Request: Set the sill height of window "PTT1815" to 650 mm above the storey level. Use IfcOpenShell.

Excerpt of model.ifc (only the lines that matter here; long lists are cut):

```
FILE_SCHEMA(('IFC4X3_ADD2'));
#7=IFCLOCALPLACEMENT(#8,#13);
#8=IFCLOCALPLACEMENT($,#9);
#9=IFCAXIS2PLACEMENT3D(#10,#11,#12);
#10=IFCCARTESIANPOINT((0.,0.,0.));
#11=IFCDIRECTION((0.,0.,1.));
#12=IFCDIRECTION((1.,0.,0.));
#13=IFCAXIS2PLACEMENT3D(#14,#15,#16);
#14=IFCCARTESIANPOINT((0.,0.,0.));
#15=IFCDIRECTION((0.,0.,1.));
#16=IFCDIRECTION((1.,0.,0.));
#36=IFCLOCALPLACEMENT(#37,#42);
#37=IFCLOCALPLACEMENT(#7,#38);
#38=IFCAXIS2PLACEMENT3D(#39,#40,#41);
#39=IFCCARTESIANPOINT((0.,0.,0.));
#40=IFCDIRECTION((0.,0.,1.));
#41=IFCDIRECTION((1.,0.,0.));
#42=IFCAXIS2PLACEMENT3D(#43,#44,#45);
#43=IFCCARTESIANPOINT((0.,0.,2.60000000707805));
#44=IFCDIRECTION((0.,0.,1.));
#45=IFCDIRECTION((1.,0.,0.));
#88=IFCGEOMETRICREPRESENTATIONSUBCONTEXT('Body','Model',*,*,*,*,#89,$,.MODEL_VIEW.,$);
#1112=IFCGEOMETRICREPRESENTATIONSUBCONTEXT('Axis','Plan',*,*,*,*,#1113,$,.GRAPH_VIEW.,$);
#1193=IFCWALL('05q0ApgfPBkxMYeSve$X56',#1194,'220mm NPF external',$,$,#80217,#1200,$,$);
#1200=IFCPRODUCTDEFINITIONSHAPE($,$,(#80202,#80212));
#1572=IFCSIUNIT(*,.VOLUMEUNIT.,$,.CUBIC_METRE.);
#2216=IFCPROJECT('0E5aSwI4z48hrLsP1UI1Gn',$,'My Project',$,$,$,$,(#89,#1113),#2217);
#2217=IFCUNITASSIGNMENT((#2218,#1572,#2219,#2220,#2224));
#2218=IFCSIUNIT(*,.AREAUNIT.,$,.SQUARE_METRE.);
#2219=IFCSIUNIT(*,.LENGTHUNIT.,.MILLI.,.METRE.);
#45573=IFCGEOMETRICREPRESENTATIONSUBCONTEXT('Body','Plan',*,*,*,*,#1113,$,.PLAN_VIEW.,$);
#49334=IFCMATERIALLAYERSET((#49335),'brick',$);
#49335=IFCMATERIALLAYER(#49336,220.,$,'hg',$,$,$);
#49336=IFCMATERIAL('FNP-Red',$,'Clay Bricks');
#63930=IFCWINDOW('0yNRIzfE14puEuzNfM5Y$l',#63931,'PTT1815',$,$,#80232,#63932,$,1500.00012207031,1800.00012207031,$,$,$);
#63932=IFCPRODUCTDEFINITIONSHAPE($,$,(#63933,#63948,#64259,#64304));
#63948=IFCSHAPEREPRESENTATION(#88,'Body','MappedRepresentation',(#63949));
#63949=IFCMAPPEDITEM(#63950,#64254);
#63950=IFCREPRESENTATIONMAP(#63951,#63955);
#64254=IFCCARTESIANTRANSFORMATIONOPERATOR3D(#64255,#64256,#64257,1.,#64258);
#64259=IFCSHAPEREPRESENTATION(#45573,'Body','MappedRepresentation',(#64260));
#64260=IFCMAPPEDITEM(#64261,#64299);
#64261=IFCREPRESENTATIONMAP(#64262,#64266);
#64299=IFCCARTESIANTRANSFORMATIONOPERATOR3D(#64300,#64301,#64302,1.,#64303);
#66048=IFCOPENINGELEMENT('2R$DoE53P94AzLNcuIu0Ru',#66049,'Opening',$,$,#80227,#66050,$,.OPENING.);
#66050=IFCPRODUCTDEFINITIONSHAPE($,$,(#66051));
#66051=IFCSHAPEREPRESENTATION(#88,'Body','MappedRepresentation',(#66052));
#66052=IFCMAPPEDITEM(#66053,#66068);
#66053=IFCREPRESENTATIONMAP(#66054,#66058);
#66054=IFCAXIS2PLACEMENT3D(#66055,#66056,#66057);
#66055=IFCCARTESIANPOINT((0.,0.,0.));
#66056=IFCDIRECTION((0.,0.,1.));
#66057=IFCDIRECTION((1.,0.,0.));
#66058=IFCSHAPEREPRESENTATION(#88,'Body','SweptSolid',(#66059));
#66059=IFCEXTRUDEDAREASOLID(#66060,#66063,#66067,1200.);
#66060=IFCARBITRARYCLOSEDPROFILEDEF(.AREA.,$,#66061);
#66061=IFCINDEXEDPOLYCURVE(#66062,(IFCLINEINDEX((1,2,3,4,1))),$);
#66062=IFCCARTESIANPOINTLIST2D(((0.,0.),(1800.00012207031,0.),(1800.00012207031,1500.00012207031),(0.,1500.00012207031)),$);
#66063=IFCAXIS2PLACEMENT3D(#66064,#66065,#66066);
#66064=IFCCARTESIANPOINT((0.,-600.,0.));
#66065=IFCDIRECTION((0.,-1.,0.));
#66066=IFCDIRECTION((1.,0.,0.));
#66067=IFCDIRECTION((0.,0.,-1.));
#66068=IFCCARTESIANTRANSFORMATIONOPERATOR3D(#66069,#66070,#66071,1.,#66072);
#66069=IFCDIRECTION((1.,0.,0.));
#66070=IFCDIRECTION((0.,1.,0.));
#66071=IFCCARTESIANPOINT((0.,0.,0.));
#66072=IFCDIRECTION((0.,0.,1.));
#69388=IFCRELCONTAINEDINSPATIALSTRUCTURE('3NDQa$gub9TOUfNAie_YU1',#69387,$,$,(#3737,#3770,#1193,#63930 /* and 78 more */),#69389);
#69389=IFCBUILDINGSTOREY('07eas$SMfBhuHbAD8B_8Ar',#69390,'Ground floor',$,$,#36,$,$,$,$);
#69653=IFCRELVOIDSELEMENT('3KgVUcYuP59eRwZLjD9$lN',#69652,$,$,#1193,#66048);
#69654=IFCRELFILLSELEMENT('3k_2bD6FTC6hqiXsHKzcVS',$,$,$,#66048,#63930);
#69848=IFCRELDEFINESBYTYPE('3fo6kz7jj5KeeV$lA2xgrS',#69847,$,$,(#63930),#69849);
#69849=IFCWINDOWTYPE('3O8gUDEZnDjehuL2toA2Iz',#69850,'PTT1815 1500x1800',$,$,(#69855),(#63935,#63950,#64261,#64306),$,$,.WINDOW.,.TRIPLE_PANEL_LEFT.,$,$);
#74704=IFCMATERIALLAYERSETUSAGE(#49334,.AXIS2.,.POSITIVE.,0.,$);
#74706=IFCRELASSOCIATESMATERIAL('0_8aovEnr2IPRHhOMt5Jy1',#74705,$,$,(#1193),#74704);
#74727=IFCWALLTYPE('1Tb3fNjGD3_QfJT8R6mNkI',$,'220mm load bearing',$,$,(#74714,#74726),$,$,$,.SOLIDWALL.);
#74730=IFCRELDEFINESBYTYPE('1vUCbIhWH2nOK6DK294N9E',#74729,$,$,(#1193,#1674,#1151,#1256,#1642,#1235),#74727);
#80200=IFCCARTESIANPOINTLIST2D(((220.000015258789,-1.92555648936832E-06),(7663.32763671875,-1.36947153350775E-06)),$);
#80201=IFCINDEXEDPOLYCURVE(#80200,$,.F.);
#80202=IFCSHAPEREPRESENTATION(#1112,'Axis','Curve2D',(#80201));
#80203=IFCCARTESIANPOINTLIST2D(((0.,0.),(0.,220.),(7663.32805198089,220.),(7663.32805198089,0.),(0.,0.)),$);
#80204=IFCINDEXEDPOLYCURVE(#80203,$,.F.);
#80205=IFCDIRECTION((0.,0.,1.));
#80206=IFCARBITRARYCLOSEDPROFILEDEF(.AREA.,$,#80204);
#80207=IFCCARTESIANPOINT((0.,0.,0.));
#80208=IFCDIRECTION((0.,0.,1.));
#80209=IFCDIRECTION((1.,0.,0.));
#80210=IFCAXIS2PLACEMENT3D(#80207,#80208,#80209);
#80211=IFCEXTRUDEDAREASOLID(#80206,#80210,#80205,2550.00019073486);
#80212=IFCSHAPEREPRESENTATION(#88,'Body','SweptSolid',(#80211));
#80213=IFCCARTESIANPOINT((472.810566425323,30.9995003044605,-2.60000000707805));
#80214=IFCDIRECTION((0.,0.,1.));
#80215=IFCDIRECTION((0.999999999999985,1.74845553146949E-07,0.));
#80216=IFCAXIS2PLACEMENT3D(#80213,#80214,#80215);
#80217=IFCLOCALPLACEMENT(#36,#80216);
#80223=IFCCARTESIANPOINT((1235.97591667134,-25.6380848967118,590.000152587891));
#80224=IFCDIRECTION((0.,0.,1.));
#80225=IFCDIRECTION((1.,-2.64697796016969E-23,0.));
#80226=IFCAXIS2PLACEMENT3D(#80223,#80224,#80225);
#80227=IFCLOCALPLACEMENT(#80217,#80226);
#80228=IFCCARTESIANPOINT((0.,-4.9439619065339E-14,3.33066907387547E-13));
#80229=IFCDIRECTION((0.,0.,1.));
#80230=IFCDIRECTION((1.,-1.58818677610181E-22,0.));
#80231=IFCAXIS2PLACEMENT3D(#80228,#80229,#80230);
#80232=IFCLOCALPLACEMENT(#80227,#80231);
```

```python
import numpy as np
import ifcopenshell
import ifcopenshell.api.geometry
import ifcopenshell.geom
import ifcopenshell.util.element
import ifcopenshell.util.placement
import ifcopenshell.util.shape
import ifcopenshell.util.unit

model = ifcopenshell.open("model.ifc")
unit_scale = ifcopenshell.util.unit.calculate_unit_scale(model)

window = model.by_id(63930)
opening = window.FillsVoids[0].RelatingOpeningElement
storey = ifcopenshell.util.element.get_container(window, ifc_class="IfcBuildingStorey")
level = ifcopenshell.util.placement.get_local_placement(storey.ObjectPlacement)[2, 3]

# The opening's origin need not be at the sill, so measure its lowest point.
shape = ifcopenshell.geom.create_shape(ifcopenshell.geom.settings(), opening)
bottom = ifcopenshell.util.shape.get_shape_bottom_elevation(shape, shape.geometry) / unit_scale
dz = level + 0.65 / unit_scale - bottom

shift = np.array([0.0, 0.0, dz])
# The window is placed relative to its opening, so it follows when the opening moves.
matrix = ifcopenshell.util.placement.get_local_placement(opening.ObjectPlacement)
matrix[:3, 3] += shift
ifcopenshell.api.geometry.edit_object_placement(
    model, product=opening, matrix=matrix, is_si=False, should_transform_children=True
)

print(f"moved by {dz * unit_scale:+.3f} m")

model.write("model_edited.ifc")
```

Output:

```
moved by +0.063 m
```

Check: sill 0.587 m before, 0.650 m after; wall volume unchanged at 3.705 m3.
